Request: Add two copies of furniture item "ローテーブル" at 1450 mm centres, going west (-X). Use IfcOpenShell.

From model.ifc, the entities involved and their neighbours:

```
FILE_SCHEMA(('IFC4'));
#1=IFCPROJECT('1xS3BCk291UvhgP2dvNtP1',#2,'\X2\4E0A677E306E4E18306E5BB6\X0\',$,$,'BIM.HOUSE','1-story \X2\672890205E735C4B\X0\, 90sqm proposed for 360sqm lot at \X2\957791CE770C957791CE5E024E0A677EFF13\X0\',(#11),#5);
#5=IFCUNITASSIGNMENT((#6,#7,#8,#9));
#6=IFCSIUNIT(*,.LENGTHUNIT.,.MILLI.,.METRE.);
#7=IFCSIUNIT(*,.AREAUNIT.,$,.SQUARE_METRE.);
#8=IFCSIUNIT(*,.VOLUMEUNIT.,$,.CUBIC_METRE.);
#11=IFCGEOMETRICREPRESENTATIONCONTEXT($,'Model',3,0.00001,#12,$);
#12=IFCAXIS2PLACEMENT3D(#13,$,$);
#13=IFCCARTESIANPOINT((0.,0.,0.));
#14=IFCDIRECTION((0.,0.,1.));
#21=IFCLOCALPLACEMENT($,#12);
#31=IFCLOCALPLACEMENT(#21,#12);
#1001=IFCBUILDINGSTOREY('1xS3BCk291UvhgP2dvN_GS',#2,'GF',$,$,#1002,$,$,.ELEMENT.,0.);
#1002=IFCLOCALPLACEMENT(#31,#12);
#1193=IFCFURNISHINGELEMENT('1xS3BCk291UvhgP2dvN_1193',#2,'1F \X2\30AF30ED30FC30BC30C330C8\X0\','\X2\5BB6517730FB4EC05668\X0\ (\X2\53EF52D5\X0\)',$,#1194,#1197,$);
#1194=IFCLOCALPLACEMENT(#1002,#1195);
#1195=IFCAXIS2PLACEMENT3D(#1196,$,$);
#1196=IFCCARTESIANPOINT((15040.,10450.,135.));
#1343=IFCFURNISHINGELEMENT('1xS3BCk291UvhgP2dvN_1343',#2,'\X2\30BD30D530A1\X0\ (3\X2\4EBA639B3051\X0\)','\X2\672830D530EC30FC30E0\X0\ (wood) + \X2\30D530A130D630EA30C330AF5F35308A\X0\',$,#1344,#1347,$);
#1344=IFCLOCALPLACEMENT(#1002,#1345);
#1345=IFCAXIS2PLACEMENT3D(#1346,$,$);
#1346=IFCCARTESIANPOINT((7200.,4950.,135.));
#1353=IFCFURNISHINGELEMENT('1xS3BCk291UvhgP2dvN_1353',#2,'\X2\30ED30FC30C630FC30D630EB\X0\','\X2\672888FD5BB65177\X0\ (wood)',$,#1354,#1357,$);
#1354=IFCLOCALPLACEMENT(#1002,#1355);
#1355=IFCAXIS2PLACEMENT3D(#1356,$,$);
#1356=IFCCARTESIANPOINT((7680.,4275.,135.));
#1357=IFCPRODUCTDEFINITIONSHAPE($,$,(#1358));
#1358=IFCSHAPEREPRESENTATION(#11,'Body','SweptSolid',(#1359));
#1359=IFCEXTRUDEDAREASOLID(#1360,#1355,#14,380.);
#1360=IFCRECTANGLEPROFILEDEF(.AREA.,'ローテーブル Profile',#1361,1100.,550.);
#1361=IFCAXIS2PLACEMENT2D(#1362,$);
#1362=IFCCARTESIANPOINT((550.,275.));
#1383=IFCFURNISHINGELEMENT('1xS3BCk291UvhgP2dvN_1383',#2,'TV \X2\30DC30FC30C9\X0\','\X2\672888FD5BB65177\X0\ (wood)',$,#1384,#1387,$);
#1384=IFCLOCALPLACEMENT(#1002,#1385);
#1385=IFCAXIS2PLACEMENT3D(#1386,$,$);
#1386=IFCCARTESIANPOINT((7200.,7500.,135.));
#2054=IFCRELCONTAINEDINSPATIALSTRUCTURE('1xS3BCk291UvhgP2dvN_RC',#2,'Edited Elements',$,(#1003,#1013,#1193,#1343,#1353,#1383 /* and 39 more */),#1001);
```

```python
import numpy as np
import ifcopenshell
import ifcopenshell.api.geometry
import ifcopenshell.api.root
import ifcopenshell.util.element
import ifcopenshell.util.placement
import ifcopenshell.util.unit

model = ifcopenshell.open("model.ifc")
unit_scale = ifcopenshell.util.unit.calculate_unit_scale(model)


def reuse_history(source, copy):
    """copy_class also copies each property set's owner history, people and application; keep the originals."""
    for rel in copy.IsDefinedBy:
        if rel.is_a("IfcRelDefinesByProperties") and (history := rel.RelatingPropertyDefinition.OwnerHistory):
            rel.RelatingPropertyDefinition.OwnerHistory = source.OwnerHistory
            ifcopenshell.util.element.remove_deep2(model, history)


source = model.by_guid("1xS3BCk291UvhgP2dvN_1353")
base = ifcopenshell.util.placement.get_local_placement(source.ObjectPlacement)
step = np.array([-1.0, 0.0, 0.0]) * 1.45 / unit_scale

for i in range(1, 3):
    copy = ifcopenshell.api.root.copy_class(model, product=source)
    copy.Representation = ifcopenshell.util.element.copy_deep(
        model, source.Representation, exclude=["IfcGeometricRepresentationContext", "IfcRepresentationMap"]
    )
    reuse_history(source, copy)
    matrix = base.copy()
    matrix[:3, 3] += i * step
    print("added at", matrix[:3, 3].round(3) + 0.0)
    ifcopenshell.api.geometry.edit_object_placement(model, product=copy, matrix=matrix, is_si=False)

model.write("model-out.ifc")
```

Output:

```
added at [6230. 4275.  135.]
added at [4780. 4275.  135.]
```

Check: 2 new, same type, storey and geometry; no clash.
